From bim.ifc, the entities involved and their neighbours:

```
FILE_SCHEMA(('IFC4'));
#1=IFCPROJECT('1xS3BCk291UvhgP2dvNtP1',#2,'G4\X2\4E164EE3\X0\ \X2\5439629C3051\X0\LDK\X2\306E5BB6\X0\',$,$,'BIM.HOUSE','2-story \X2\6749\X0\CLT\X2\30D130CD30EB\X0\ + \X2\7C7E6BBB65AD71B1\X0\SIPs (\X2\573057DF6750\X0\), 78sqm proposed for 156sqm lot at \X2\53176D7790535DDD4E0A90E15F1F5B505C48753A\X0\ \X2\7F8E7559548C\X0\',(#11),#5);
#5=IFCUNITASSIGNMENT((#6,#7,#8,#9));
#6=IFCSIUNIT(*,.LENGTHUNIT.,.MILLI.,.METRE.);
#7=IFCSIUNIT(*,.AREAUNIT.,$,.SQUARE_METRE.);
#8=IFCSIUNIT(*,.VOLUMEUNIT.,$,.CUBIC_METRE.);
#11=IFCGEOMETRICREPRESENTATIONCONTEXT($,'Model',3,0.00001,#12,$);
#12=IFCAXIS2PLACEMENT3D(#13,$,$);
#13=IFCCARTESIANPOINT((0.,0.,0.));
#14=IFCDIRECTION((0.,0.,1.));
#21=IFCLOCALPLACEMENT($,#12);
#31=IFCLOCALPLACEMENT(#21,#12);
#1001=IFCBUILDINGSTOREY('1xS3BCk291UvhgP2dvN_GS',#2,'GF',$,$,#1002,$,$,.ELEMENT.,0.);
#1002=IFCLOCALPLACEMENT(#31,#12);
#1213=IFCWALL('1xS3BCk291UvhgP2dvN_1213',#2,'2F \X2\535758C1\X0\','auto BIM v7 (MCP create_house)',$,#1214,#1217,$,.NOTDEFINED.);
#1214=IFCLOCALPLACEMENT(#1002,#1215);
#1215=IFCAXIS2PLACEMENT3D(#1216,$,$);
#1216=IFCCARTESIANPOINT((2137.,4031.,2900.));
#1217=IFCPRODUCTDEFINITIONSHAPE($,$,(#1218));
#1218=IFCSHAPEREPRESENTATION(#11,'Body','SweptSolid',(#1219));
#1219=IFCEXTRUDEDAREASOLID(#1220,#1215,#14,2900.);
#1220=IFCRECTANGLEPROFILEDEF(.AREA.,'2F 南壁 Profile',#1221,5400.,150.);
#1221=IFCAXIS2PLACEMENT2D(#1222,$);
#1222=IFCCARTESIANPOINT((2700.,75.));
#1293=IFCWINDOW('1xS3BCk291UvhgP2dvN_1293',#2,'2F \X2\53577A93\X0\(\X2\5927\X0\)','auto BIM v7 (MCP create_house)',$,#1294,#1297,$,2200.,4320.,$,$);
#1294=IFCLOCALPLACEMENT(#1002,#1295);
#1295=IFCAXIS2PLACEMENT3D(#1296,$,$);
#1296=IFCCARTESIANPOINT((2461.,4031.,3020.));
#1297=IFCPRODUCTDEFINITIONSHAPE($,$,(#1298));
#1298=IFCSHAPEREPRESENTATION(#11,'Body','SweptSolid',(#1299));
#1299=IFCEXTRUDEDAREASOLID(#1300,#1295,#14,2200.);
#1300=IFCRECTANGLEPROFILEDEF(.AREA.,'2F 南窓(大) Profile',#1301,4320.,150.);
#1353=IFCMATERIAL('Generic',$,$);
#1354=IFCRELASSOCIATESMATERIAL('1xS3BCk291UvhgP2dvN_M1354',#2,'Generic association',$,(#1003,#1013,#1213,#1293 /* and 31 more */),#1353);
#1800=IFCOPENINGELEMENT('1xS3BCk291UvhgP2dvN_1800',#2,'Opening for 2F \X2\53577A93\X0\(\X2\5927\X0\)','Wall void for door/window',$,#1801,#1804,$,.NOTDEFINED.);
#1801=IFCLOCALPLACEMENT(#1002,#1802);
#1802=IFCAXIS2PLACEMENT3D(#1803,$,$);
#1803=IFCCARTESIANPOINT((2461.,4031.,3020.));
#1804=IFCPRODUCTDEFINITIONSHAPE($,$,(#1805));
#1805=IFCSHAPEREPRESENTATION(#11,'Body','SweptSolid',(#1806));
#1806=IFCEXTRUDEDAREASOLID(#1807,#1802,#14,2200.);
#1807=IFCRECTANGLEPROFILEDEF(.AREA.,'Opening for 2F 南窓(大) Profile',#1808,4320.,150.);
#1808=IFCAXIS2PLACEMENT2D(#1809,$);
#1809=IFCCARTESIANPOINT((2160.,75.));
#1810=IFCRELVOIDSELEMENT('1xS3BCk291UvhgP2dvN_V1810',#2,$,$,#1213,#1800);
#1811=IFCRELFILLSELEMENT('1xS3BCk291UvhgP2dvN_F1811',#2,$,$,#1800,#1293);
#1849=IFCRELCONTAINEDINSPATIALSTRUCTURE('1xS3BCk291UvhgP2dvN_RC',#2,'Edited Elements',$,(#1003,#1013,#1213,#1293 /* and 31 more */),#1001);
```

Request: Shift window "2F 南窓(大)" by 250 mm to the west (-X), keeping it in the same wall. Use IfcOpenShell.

```python
import ifcopenshell
import ifcopenshell.api.geometry
import ifcopenshell.util.placement
import ifcopenshell.util.unit

model = ifcopenshell.open("bim.ifc")
unit_scale = ifcopenshell.util.unit.calculate_unit_scale(model)

window = model.by_id(1293)
opening = window.FillsVoids[0].RelatingOpeningElement
wall = opening.VoidsElements[0].RelatingBuildingElement

wall_matrix = ifcopenshell.util.placement.get_local_placement(wall.ObjectPlacement)
shift = wall_matrix[:3, 0] * -0.25 / unit_scale
before = ifcopenshell.util.placement.get_local_placement(window.ObjectPlacement)[:3, 3].copy()

# The window is not placed relative to its opening, so move both.
for product in (opening, window):
    matrix = ifcopenshell.util.placement.get_local_placement(product.ObjectPlacement)
    matrix[:3, 3] += shift
    ifcopenshell.api.geometry.edit_object_placement(model, product=product, matrix=matrix, is_si=False)

after = ifcopenshell.util.placement.get_local_placement(window.ObjectPlacement)[:3, 3]
print("window moved by", (after - before).round(3) + 0.0)

model.write("bim-out.ifc")
```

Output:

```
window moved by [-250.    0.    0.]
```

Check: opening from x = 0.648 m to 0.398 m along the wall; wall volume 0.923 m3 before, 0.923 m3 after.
